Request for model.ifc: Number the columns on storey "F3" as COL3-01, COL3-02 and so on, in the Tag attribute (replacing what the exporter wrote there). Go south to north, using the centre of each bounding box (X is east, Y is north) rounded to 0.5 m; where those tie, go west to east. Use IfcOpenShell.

First a look at what the model holds.

```python
import ifcopenshell
import ifcopenshell.util.element
import ifcopenshell.util.placement

model = ifcopenshell.open("model.ifc")
print(model.schema)
storey = next(s for s in model.by_type("IfcBuildingStorey") if s.Name == "F3")
columns = [e for e in ifcopenshell.util.element.get_decomposition(storey) if e.is_a("IfcColumn")]
for e in sorted(columns, key=lambda e: e.id()):
    origin = ifcopenshell.util.placement.get_local_placement(e.ObjectPlacement)[:3, 3]
    print(e.id(), e.Tag, e.Name, origin.round(2) + 0.0, sep=" | ")
```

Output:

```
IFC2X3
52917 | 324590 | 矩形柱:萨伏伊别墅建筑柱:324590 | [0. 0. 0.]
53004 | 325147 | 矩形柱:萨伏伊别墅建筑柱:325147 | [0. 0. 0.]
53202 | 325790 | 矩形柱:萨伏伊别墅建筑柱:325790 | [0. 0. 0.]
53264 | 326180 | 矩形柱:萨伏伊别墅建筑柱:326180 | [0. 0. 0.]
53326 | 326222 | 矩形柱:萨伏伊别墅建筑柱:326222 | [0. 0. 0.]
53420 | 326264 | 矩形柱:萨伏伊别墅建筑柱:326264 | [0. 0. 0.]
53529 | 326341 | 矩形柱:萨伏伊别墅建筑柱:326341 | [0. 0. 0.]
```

```python
import ifcopenshell
import ifcopenshell.geom
import ifcopenshell.util.element
import ifcopenshell.util.shape

model = ifcopenshell.open("model.ifc")
settings = ifcopenshell.geom.settings()
settings.set("use-world-coords", True)


def centre(element):
    shape = ifcopenshell.geom.create_shape(settings, element)
    return ifcopenshell.util.shape.get_bbox_centroid(shape.geometry)


storey = next(s for s in model.by_type("IfcBuildingStorey") if s.Name == "F3")
columns = [e for e in ifcopenshell.util.element.get_decomposition(storey) if e.is_a("IfcColumn")]

# Insertion points can sit at a corner or the storey origin, so sort by the geometry (in metres).
centres = {e: centre(e) for e in columns}
columns.sort(key=lambda e: (round(centres[e][1] / 0.5), centres[e][0]))

for i, e in enumerate(columns, start=1):
    number = f"COL3-{i:02d}"
    e.Tag = number
    print(e.id(), number)

model.write("model_updated.ifc")
```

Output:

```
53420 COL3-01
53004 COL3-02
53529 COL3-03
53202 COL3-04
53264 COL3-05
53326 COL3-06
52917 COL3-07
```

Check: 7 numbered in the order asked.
